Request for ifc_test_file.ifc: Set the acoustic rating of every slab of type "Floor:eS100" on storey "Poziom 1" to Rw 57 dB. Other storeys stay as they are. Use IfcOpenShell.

First a look at what the model holds.

```python
import ifcopenshell
import ifcopenshell.util.element

model = ifcopenshell.open("ifc_test_file.ifc")
print(model.schema)
storey = next(s for s in model.by_type("IfcBuildingStorey") if s.Name == "Poziom 1")
slabs = [e for e in ifcopenshell.util.element.get_decomposition(storey) if e.is_a("IfcSlab")]
seen = {}
for e in slabs:
    element_type = ifcopenshell.util.element.get_type(e)
    key = (element_type.Name if element_type != e and element_type else None, ifcopenshell.util.element.get_pset(e, "Pset_SlabCommon", "AcousticRating"))
    seen[key] = seen.get(key, 0) + 1
for (name, value), count in sorted(seen.items(), key=str):
    print(count, "x", name, "|", value)
```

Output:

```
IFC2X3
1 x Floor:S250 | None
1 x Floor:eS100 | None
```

```python
import ifcopenshell
import ifcopenshell.api.pset
import ifcopenshell.util.element

model = ifcopenshell.open("ifc_test_file.ifc")

storey = next(s for s in model.by_type("IfcBuildingStorey") if s.Name == "Poziom 1")
slabs = [e for e in ifcopenshell.util.element.get_decomposition(storey) if e.is_a("IfcSlab")]

count = 0
for e in slabs:
    element_type = ifcopenshell.util.element.get_type(e)
    if element_type in (None, e) or element_type.Name != "Floor:eS100":
        continue
    # add_pset returns the element's existing set when there is one.
    pset = ifcopenshell.api.pset.add_pset(model, product=e, name="Pset_SlabCommon")
    ifcopenshell.api.pset.edit_pset(model, pset=pset, properties={"AcousticRating": "Rw 57 dB"})
    count += 1

print(count, "slabs updated")

model.write("ifc_test_file_updated.ifc")
```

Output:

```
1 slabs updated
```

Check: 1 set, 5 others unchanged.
